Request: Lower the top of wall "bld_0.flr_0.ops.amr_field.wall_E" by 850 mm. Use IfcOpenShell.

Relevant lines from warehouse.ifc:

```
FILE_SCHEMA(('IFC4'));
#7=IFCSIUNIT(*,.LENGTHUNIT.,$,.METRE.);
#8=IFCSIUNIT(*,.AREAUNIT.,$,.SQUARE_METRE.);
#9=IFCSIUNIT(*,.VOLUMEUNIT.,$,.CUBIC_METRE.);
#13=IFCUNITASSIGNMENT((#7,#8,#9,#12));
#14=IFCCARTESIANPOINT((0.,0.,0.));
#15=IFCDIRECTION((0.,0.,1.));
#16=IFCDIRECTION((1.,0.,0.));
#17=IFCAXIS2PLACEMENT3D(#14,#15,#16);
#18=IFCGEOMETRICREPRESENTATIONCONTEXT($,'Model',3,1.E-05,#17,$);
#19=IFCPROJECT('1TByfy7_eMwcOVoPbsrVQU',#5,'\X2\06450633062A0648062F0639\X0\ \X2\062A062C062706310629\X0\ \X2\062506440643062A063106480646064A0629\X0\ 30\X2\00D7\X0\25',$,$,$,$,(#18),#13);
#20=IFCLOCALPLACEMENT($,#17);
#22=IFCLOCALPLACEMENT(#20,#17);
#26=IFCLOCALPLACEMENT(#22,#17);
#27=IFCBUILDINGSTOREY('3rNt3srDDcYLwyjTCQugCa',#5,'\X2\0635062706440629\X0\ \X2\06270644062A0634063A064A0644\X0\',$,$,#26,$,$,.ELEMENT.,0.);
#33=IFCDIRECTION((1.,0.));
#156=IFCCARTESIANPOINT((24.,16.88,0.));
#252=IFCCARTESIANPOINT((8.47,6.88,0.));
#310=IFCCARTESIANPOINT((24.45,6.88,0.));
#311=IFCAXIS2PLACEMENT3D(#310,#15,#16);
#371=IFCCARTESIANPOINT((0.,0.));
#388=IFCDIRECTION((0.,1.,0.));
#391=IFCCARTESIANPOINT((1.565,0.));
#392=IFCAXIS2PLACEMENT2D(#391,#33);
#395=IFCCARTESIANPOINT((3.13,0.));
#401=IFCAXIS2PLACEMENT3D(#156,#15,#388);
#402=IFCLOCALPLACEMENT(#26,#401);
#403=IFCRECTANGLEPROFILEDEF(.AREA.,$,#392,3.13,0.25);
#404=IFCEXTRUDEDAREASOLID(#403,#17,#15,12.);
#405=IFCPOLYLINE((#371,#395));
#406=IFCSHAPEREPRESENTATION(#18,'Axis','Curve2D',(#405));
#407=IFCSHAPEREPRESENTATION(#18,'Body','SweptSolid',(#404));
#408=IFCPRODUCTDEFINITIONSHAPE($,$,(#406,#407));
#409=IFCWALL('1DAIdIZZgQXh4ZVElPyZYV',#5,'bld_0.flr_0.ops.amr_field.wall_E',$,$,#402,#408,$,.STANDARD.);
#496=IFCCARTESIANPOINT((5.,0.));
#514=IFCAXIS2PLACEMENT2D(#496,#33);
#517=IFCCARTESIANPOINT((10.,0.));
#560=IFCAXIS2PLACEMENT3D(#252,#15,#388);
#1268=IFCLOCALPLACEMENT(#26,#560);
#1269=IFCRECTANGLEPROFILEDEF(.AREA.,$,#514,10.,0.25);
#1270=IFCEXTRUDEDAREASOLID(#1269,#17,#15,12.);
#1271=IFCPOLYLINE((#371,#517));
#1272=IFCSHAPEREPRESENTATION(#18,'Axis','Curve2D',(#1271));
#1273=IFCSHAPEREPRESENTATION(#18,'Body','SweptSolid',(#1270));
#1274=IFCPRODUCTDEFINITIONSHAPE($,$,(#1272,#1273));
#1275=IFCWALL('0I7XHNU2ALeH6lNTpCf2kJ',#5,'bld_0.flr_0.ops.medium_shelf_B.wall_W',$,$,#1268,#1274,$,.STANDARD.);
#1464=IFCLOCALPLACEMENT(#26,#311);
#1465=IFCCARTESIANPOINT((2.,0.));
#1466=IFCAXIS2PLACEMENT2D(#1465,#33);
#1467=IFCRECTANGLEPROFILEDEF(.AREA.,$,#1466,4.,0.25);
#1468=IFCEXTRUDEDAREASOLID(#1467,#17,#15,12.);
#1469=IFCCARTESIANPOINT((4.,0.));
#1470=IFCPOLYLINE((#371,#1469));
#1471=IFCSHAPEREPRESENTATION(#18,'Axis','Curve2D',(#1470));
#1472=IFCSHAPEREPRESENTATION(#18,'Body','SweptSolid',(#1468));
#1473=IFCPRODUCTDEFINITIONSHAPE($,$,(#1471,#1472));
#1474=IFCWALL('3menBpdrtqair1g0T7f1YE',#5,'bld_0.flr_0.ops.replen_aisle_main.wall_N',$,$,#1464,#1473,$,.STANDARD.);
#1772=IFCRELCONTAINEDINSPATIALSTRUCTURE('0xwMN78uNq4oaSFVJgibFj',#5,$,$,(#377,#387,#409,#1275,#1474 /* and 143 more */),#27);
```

```python
import ifcopenshell
import ifcopenshell.geom
import ifcopenshell.util.shape
import ifcopenshell.util.unit

model = ifcopenshell.open("warehouse.ifc")
unit_scale = ifcopenshell.util.unit.calculate_unit_scale(model)
settings = ifcopenshell.geom.settings()


def volume(element):
    """Net volume in cubic metres, openings subtracted."""
    shape = ifcopenshell.geom.create_shape(settings, element)
    return ifcopenshell.util.shape.get_volume(shape.geometry)


wall = model.by_guid("1DAIdIZZgQXh4ZVElPyZYV")
before = volume(wall)

body = next(r for r in wall.Representation.Representations if r.RepresentationIdentifier == "Body")
solid = body.Items[0]
old_height = solid.Depth
solid.Depth -= 0.85 / unit_scale
after = volume(wall)

print(f"height {old_height:g} -> {solid.Depth:g}, volume {before:.3f} -> {after:.3f} m3")

model.write("warehouse_edited.ifc")
```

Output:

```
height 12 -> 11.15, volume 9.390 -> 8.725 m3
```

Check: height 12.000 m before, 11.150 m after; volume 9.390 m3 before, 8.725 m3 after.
